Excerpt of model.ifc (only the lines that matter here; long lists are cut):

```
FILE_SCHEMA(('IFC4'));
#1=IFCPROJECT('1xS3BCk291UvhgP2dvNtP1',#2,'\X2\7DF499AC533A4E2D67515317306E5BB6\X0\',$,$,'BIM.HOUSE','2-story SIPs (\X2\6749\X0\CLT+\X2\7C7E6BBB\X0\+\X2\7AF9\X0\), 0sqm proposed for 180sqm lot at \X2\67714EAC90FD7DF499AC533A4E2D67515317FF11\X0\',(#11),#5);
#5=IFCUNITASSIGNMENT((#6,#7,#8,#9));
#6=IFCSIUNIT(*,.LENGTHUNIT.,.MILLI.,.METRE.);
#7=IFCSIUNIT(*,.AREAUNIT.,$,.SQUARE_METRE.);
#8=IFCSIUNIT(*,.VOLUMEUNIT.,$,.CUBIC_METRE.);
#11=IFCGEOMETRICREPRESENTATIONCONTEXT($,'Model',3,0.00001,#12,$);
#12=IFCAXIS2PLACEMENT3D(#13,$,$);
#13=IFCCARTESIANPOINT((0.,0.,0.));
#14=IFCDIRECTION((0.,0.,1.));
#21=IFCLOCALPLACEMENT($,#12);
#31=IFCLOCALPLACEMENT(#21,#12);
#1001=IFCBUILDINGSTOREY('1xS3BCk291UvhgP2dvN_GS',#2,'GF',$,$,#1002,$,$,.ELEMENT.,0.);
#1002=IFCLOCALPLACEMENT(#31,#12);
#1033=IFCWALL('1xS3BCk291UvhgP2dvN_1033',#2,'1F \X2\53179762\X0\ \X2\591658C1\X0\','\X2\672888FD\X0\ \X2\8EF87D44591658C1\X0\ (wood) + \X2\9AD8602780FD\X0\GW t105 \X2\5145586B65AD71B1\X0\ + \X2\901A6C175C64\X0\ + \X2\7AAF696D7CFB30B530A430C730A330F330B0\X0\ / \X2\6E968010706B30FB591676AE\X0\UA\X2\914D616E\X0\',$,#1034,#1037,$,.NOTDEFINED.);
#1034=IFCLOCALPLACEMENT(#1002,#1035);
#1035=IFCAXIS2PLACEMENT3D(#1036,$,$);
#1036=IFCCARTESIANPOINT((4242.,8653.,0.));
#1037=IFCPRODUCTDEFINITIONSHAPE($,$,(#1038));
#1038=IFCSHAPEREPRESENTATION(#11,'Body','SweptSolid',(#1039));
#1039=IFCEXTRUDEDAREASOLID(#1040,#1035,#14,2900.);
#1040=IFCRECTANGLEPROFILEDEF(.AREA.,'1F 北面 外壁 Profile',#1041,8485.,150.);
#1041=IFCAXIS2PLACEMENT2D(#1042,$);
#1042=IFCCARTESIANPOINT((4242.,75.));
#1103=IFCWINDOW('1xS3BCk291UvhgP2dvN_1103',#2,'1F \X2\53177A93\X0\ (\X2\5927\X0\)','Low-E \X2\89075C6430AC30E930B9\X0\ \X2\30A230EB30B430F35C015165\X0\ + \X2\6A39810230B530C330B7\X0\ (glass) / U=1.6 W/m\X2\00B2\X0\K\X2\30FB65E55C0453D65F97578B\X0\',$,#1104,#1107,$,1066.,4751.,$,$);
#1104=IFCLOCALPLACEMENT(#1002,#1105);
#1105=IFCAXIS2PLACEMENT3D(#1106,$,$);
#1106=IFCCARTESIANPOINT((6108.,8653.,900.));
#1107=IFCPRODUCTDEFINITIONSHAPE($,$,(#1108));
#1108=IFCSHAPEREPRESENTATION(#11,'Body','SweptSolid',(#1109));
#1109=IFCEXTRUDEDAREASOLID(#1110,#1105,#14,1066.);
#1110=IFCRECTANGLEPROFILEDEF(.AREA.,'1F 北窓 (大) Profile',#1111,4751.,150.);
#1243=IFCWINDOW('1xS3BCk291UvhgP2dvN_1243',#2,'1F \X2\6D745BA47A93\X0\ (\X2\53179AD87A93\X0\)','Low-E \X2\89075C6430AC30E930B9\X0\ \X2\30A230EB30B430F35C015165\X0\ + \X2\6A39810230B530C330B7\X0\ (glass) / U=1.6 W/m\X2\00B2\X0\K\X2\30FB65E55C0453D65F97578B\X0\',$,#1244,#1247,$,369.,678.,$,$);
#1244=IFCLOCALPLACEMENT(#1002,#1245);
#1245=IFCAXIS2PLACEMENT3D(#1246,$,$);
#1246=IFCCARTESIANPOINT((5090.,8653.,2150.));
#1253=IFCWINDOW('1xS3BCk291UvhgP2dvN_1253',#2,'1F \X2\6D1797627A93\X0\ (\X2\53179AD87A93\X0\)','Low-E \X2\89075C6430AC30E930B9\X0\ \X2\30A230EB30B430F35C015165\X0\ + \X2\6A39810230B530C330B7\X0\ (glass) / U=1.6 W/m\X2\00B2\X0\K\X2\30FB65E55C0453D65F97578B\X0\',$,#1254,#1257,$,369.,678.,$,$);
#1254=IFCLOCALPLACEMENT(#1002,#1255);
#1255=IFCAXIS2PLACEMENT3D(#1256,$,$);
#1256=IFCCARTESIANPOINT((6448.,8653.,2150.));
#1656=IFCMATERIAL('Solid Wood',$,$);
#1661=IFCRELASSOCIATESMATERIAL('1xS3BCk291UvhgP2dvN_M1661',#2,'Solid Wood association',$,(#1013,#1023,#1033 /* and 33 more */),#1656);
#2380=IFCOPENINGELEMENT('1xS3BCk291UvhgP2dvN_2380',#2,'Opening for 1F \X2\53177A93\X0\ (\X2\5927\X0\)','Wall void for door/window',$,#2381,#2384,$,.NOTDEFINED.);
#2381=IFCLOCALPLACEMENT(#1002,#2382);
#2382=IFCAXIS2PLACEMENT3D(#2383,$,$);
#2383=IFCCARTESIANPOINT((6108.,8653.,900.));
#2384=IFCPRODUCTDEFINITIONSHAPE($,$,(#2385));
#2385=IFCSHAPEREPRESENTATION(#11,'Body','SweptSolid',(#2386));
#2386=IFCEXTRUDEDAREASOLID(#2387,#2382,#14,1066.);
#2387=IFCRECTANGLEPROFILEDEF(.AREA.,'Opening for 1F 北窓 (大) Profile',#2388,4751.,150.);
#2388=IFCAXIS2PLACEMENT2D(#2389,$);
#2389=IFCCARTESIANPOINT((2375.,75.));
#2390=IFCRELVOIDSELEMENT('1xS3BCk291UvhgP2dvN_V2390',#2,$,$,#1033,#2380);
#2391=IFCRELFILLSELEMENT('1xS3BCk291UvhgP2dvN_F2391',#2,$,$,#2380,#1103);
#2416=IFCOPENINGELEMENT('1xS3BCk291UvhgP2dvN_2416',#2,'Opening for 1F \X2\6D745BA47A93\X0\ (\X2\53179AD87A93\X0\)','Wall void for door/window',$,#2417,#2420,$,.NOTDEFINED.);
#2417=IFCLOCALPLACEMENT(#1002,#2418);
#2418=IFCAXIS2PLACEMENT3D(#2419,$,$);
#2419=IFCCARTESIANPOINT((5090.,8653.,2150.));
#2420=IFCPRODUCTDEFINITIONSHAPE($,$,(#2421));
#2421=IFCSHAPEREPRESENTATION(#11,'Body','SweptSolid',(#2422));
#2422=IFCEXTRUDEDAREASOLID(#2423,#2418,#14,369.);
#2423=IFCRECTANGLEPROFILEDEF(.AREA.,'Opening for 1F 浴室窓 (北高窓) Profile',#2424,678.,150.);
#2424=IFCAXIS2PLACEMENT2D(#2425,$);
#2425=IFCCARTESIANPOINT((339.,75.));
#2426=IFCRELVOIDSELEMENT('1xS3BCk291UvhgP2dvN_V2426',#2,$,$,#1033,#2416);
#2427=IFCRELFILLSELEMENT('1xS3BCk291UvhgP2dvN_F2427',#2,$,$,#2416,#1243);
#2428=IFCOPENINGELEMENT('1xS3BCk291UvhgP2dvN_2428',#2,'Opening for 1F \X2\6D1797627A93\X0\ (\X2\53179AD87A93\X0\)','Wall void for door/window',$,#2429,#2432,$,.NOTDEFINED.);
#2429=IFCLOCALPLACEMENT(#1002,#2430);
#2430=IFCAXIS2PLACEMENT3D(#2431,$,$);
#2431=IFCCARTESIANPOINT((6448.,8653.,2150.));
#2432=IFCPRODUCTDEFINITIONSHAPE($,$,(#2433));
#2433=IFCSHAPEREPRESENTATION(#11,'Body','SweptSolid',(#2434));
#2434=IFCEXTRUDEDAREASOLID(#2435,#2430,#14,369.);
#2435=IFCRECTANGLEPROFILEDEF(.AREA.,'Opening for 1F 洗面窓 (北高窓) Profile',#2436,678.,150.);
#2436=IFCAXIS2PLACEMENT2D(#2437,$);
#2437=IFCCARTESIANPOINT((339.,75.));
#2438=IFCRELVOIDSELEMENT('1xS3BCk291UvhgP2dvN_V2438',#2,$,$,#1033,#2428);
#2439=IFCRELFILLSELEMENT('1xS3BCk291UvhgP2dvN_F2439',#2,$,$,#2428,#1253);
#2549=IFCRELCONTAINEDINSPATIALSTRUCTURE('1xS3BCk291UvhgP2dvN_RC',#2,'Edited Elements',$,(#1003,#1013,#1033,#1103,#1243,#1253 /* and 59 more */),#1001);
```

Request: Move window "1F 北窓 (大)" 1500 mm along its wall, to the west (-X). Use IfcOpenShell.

```python
import ifcopenshell
import ifcopenshell.api.geometry
import ifcopenshell.util.placement

model = ifcopenshell.open("model.ifc")

window = model.by_guid("1xS3BCk291UvhgP2dvN_1103")
opening = window.FillsVoids[0].RelatingOpeningElement
wall = opening.VoidsElements[0].RelatingBuildingElement

wall_matrix = ifcopenshell.util.placement.get_local_placement(wall.ObjectPlacement)
shift = wall_matrix[:3, 0] * -1500.0
before = ifcopenshell.util.placement.get_local_placement(window.ObjectPlacement)[:3, 3].copy()

# The window is not placed relative to its opening, so move both.
for product in (opening, window):
    matrix = ifcopenshell.util.placement.get_local_placement(product.ObjectPlacement)
    matrix[:3, 3] += shift
    ifcopenshell.api.geometry.edit_object_placement(model, product=product, matrix=matrix, is_si=False)

after = ifcopenshell.util.placement.get_local_placement(window.ObjectPlacement)[:3, 3]
print("window moved by", (after - before).round(3) + 0.0)

model.write("model-out.ifc")
```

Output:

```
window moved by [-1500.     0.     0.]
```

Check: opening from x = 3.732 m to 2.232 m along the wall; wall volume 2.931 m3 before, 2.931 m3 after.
